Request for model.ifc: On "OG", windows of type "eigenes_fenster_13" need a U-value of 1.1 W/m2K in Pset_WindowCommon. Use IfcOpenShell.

First a look at what the model holds.

```python
import ifcopenshell
import ifcopenshell.util.element

model = ifcopenshell.open("model.ifc")
print(model.schema)
storey = next(s for s in model.by_type("IfcBuildingStorey") if s.Name == "OG")
windows = [e for e in ifcopenshell.util.element.get_decomposition(storey) if e.is_a("IfcWindow")]
seen = {}
for e in windows:
    element_type = ifcopenshell.util.element.get_type(e)
    key = (element_type.Name if element_type != e and element_type else None, ifcopenshell.util.element.get_pset(e, "Pset_WindowCommon", "ThermalTransmittance"))
    seen[key] = seen.get(key, 0) + 1
for (name, value), count in sorted(seen.items(), key=str):
    print(count, "x", name, "|", value)
```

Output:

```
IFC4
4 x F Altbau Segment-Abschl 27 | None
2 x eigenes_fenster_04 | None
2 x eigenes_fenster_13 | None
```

```python
import ifcopenshell
import ifcopenshell.api.pset
import ifcopenshell.util.element

model = ifcopenshell.open("model.ifc")

storey = next(s for s in model.by_type("IfcBuildingStorey") if s.Name == "OG")
windows = [e for e in ifcopenshell.util.element.get_decomposition(storey) if e.is_a("IfcWindow")]

count = 0
for e in windows:
    element_type = ifcopenshell.util.element.get_type(e)
    if element_type in (None, e) or element_type.Name != "eigenes_fenster_13":
        continue
    # add_pset returns the element's existing set when there is one.
    pset = ifcopenshell.api.pset.add_pset(model, product=e, name="Pset_WindowCommon")
    ifcopenshell.api.pset.edit_pset(model, pset=pset, properties={"ThermalTransmittance": 1.1})
    count += 1

print(count, "windows updated")

model.write("model_edited.ifc")
```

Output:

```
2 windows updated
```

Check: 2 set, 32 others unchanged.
